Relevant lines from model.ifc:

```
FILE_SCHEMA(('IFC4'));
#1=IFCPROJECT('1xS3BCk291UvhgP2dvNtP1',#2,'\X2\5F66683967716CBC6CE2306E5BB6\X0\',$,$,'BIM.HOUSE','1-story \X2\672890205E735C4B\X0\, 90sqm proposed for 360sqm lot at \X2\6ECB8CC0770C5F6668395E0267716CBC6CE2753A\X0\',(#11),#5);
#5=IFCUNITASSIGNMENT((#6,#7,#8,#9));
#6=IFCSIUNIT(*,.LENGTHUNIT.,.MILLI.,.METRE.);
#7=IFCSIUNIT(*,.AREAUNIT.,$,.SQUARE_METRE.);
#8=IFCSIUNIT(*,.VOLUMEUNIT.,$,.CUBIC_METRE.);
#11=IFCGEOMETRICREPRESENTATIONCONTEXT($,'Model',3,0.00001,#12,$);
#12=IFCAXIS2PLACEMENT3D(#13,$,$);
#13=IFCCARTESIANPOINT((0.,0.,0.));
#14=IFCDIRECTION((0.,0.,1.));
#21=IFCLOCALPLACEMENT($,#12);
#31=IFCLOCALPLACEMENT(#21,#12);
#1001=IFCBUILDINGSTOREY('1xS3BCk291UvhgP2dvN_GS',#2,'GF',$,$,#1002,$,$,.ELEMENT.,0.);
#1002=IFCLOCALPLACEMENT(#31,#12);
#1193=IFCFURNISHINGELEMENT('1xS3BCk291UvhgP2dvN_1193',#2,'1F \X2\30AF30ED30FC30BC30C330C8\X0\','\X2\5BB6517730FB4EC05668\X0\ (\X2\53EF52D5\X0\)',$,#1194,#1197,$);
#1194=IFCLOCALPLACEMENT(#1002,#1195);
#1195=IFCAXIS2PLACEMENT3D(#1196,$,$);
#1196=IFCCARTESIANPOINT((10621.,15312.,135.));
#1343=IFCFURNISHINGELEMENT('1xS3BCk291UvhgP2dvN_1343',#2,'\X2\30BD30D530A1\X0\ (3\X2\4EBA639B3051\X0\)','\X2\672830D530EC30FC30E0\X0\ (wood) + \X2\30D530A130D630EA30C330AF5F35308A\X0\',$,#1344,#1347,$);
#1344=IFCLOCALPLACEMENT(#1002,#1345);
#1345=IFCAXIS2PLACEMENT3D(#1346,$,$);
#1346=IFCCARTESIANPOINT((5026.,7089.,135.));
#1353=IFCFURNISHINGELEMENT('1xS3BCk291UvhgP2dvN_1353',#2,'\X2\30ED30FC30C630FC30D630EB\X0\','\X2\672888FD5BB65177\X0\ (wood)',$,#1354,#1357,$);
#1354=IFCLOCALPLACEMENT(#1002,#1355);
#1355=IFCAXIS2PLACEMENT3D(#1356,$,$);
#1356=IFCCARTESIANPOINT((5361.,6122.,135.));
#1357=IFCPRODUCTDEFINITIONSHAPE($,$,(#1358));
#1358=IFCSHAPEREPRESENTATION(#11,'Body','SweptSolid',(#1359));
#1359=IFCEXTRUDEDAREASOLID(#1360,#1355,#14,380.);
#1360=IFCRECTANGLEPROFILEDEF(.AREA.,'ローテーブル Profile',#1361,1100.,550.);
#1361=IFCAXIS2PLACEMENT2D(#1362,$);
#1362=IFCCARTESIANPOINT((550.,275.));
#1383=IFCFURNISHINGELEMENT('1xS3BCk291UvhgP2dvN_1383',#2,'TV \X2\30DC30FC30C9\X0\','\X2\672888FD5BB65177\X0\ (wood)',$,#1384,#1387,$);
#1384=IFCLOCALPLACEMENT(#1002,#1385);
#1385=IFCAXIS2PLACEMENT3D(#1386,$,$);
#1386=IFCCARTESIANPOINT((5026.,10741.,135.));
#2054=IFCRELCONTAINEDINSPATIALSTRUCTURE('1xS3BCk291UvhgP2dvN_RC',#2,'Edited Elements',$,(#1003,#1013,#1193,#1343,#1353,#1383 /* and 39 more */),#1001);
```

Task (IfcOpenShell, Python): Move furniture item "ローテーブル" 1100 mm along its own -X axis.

```python
import ifcopenshell
import ifcopenshell.api.geometry
import ifcopenshell.util.placement

model = ifcopenshell.open("model.ifc")

item = model.by_guid("1xS3BCk291UvhgP2dvN_1353")
matrix = ifcopenshell.util.placement.get_local_placement(item.ObjectPlacement)
matrix[:3, 3] -= matrix[:3, 0] * 1100.0
ifcopenshell.api.geometry.edit_object_placement(model, product=item, matrix=matrix, is_si=False)

print(ifcopenshell.util.placement.get_local_placement(item.ObjectPlacement).round(3) + 0.0)

model.write("model-out.ifc")
```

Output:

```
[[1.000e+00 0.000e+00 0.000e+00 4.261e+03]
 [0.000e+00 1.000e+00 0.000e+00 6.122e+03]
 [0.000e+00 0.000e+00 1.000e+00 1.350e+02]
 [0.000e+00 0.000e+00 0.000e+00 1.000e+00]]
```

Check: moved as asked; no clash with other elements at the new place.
